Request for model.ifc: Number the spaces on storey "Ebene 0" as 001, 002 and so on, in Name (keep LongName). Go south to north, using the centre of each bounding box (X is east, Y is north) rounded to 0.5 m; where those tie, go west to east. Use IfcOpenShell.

First a look at what the model holds.

```python
import ifcopenshell
import ifcopenshell.util.element
import ifcopenshell.util.placement

model = ifcopenshell.open("model.ifc")
print(model.schema)
storey = next(s for s in model.by_type("IfcBuildingStorey") if s.Name == "Ebene 0")
spaces = [e for e in ifcopenshell.util.element.get_decomposition(storey) if e.is_a("IfcSpace")]
for e in sorted(spaces, key=lambda e: e.id()):
    origin = ifcopenshell.util.placement.get_local_placement(e.ObjectPlacement)[:3, 3]
    print(e.id(), e.Name, e.LongName, origin.round(2) + 0.0, sep=" | ")
```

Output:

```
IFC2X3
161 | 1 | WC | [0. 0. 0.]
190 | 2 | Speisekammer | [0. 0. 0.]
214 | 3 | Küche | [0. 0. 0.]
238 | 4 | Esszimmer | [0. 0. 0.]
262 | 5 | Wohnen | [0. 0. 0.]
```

```python
import ifcopenshell
import ifcopenshell.geom
import ifcopenshell.util.element
import ifcopenshell.util.shape

model = ifcopenshell.open("model.ifc")
settings = ifcopenshell.geom.settings()
settings.set("use-world-coords", True)


def centre(element):
    shape = ifcopenshell.geom.create_shape(settings, element)
    return ifcopenshell.util.shape.get_bbox_centroid(shape.geometry)


storey = next(s for s in model.by_type("IfcBuildingStorey") if s.Name == "Ebene 0")
spaces = [e for e in ifcopenshell.util.element.get_decomposition(storey) if e.is_a("IfcSpace")]

# Insertion points can sit at a corner or the storey origin, so sort by the geometry (in metres).
centres = {e: centre(e) for e in spaces}
spaces.sort(key=lambda e: (round(centres[e][1] / 0.5), centres[e][0]))

for i, e in enumerate(spaces, start=1):
    number = f"0{i:02d}"
    e.Name = number
    print(e.id(), number)

model.write("model-out.ifc")
```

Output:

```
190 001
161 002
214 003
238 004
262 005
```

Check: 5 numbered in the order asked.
